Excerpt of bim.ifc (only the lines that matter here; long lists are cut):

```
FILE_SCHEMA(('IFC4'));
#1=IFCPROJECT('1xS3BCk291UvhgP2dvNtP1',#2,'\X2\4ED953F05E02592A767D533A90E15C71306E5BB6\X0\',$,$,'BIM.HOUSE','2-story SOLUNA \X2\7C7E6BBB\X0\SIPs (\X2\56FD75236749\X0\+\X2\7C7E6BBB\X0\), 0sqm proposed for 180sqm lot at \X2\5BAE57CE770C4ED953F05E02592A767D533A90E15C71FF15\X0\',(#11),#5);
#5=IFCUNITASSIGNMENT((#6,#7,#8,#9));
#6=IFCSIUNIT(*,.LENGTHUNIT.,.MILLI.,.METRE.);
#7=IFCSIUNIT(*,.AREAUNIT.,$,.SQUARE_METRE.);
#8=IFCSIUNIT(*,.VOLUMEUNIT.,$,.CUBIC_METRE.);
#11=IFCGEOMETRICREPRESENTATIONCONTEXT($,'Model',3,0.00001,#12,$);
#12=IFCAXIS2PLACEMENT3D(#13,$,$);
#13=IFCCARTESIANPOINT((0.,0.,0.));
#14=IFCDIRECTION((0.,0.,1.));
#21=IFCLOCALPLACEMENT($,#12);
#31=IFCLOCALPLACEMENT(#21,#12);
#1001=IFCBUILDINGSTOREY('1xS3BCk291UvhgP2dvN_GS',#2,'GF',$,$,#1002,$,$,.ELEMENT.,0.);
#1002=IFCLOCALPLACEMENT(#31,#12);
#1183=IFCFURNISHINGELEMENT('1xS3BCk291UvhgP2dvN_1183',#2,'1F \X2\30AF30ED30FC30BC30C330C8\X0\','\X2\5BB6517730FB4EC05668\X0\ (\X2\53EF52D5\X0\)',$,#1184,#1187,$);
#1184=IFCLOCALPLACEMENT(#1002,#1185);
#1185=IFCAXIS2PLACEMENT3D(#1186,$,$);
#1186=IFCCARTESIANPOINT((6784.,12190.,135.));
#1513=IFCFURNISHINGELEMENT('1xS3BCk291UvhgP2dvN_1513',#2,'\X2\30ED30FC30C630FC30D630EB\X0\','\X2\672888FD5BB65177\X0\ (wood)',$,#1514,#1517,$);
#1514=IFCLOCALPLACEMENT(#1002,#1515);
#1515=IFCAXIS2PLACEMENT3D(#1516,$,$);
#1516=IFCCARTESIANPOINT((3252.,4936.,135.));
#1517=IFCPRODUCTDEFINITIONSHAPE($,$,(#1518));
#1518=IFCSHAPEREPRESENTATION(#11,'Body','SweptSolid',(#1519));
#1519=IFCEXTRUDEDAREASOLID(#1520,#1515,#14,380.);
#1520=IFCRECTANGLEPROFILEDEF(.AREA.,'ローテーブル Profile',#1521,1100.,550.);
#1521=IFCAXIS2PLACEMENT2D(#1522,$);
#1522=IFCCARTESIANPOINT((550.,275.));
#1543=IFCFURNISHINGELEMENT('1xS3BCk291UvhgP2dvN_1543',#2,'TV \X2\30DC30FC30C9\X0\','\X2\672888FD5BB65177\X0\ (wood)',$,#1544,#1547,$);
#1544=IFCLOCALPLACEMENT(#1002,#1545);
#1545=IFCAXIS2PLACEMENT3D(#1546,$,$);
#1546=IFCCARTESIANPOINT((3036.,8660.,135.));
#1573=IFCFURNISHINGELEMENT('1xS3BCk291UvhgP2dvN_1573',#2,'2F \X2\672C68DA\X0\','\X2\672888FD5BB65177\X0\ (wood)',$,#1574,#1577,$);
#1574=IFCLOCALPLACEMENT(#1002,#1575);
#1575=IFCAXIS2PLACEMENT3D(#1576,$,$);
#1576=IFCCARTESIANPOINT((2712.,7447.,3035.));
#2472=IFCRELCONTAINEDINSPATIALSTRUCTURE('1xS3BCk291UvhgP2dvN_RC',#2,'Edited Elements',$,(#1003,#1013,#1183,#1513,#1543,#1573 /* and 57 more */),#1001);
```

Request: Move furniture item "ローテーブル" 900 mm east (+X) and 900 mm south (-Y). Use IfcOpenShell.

```python
import ifcopenshell
import ifcopenshell.api.geometry
import ifcopenshell.util.placement
import ifcopenshell.util.unit

model = ifcopenshell.open("bim.ifc")
unit_scale = ifcopenshell.util.unit.calculate_unit_scale(model)

item = model.by_guid("1xS3BCk291UvhgP2dvN_1513")
matrix = ifcopenshell.util.placement.get_local_placement(item.ObjectPlacement)
matrix[0, 3] += 0.9 / unit_scale
matrix[1, 3] -= 0.9 / unit_scale
ifcopenshell.api.geometry.edit_object_placement(model, product=item, matrix=matrix, is_si=False)

print(ifcopenshell.util.placement.get_local_placement(item.ObjectPlacement).round(3) + 0.0)

model.write("bim_edited.ifc")
```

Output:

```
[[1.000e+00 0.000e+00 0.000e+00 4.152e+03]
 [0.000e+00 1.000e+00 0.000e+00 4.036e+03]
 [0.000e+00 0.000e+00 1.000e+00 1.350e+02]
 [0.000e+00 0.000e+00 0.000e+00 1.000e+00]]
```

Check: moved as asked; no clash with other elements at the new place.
